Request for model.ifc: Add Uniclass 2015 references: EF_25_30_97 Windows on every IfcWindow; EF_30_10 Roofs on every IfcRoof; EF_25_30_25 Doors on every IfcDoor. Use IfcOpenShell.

First a look at what the model holds.

```python
import ifcopenshell

model = ifcopenshell.open("model.ifc")
print(model.schema)
print("classifications:", [c.Name for c in model.by_type("IfcClassification")])
for ifc_class in ("IfcDoor", "IfcRoof", "IfcStair", "IfcWall", "IfcWindow"):
    print(ifc_class, len(model.by_type(ifc_class)))
```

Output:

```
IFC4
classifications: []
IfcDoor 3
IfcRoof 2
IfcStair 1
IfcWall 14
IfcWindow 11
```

```python
import ifcopenshell
import ifcopenshell.api.classification

model = ifcopenshell.open("model.ifc")

system = ifcopenshell.api.classification.add_classification(model, classification="Uniclass 2015")

codes = {
    "IfcWindow": ("EF_25_30_97", "Windows"),
    "IfcRoof": ("EF_30_10", "Roofs"),
    "IfcDoor": ("EF_25_30_25", "Doors"),
}
for ifc_class, (code, name) in codes.items():
    products = model.by_type(ifc_class)
    ifcopenshell.api.classification.add_reference(
        model, products=products, classification=system, identification=code, name=name
    )
    print(code, len(products))

model.write("model_edited.ifc")
```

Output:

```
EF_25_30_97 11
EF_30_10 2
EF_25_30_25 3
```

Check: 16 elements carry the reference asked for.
